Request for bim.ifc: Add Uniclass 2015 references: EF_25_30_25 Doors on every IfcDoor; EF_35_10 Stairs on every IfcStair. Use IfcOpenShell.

First a look at what the model holds.

```python
import ifcopenshell

model = ifcopenshell.open("bim.ifc")
print(model.schema)
print("classifications:", [c.Name for c in model.by_type("IfcClassification")])
for ifc_class in ("IfcDoor", "IfcRoof", "IfcStair", "IfcWall", "IfcWindow"):
    print(ifc_class, len(model.by_type(ifc_class)))
```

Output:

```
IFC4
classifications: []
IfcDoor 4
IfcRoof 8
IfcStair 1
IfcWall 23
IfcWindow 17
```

```python
import ifcopenshell
import ifcopenshell.api.classification

model = ifcopenshell.open("bim.ifc")

system = ifcopenshell.api.classification.add_classification(model, classification="Uniclass 2015")

codes = {
    "IfcDoor": ("EF_25_30_25", "Doors"),
    "IfcStair": ("EF_35_10", "Stairs"),
}
for ifc_class, (code, name) in codes.items():
    products = model.by_type(ifc_class)
    ifcopenshell.api.classification.add_reference(
        model, products=products, classification=system, identification=code, name=name
    )
    print(code, len(products))

model.write("bim_updated.ifc")
```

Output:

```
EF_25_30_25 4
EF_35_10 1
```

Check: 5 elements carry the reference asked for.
